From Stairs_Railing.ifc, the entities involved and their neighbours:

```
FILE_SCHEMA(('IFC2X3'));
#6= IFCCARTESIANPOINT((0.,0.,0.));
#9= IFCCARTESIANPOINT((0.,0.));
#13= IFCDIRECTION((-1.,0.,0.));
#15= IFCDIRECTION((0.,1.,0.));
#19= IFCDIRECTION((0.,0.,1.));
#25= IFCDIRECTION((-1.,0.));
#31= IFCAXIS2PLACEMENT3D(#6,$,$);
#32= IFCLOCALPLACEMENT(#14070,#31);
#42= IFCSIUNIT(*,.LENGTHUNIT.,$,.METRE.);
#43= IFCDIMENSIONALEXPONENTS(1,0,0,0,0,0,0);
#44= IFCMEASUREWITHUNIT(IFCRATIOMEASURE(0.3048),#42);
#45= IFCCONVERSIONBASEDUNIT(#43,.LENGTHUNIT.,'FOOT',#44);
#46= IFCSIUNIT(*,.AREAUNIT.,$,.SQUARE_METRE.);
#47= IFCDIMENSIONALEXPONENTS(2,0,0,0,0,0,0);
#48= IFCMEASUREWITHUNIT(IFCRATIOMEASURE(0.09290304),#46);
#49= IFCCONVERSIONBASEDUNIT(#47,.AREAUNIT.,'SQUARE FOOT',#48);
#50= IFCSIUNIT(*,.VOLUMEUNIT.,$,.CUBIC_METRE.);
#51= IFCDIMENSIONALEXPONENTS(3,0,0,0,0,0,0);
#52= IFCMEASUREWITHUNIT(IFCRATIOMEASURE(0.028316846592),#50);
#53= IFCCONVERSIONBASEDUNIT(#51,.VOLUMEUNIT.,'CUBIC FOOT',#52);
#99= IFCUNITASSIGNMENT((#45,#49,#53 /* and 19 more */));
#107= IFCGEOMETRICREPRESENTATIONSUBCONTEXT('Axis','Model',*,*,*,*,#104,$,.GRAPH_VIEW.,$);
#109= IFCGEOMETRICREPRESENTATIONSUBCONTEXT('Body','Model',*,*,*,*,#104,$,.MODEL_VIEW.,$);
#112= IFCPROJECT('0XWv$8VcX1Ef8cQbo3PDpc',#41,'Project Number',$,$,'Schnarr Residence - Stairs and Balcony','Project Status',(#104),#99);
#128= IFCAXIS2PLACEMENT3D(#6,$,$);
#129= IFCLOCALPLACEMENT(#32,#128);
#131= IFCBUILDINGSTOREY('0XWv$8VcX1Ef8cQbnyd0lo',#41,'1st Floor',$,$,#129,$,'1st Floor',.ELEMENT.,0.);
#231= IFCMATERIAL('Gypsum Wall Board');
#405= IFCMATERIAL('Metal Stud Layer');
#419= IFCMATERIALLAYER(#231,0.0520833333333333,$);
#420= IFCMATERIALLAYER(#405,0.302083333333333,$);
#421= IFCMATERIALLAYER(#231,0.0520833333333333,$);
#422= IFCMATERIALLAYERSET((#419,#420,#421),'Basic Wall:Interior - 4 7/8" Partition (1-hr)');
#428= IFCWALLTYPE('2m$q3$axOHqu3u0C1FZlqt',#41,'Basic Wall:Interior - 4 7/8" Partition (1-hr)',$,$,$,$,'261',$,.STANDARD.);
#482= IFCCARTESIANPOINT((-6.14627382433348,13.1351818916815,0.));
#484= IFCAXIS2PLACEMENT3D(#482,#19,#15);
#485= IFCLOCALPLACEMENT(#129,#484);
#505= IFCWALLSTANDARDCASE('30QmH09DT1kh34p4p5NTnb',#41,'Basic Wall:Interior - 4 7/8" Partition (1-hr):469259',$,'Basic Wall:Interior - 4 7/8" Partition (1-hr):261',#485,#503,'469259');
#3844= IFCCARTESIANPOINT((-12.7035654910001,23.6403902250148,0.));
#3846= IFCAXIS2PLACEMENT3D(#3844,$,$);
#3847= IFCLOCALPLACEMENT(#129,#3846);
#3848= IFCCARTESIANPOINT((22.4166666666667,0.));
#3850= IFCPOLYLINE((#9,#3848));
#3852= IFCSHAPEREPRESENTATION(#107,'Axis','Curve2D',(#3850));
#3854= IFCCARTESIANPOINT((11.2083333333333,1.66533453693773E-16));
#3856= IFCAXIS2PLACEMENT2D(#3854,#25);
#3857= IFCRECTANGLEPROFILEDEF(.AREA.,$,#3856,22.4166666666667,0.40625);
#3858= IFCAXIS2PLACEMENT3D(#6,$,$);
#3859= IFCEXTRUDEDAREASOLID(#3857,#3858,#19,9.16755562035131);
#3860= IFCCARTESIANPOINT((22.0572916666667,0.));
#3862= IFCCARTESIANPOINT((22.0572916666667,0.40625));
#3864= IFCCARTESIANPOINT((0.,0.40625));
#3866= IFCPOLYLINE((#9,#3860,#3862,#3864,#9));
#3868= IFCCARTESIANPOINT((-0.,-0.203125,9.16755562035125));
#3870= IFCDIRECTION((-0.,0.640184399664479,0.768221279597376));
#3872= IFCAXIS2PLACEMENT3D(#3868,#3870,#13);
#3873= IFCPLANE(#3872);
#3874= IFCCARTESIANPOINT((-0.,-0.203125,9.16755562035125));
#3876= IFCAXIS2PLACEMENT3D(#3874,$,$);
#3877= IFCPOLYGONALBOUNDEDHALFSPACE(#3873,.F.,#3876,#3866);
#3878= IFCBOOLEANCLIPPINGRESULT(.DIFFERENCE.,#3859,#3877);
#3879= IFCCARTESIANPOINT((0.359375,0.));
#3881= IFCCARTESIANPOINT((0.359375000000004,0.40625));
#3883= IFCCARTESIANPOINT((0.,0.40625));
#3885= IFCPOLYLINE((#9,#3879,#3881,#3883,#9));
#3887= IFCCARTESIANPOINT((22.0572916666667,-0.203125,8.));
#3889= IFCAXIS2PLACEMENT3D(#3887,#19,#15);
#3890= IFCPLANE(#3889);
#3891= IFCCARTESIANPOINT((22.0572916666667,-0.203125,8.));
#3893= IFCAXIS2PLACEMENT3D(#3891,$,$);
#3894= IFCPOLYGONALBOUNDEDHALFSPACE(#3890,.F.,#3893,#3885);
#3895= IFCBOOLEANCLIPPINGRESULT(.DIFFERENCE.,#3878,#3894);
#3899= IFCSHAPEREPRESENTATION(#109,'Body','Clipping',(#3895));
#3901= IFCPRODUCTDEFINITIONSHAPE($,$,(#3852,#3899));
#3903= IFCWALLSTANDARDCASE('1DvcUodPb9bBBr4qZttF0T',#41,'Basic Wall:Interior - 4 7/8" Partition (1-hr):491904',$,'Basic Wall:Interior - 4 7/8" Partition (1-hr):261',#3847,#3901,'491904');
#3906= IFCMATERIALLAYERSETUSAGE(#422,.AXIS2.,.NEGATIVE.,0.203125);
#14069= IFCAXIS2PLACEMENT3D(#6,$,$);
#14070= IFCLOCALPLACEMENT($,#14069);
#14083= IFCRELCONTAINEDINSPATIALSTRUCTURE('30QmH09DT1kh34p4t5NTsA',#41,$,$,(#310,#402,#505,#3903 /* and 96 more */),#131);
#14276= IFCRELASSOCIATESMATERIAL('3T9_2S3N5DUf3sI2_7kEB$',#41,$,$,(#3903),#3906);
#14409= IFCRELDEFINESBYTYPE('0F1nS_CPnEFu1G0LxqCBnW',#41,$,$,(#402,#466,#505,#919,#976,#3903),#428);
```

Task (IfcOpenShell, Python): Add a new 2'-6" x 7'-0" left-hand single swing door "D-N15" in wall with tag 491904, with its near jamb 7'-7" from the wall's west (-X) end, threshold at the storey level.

```python
import numpy as np
import ifcopenshell
import ifcopenshell.api.feature
import ifcopenshell.api.geometry
import ifcopenshell.api.root
import ifcopenshell.api.spatial
import ifcopenshell.api.type
import ifcopenshell.geom
import ifcopenshell.util.element
import ifcopenshell.util.placement
import ifcopenshell.util.representation
import ifcopenshell.util.shape
import ifcopenshell.util.unit

model = ifcopenshell.open("Stairs_Railing.ifc")
unit_scale = ifcopenshell.util.unit.calculate_unit_scale(model)
settings = ifcopenshell.geom.settings()


def volume(element):
    """Net volume in cubic metres, openings subtracted."""
    shape = ifcopenshell.geom.create_shape(settings, element)
    return ifcopenshell.util.shape.get_volume(shape.geometry)


wall = model.by_guid("1DvcUodPb9bBBr4qZttF0T")
storey = ifcopenshell.util.element.get_container(wall, ifc_class="IfcBuildingStorey")
context = ifcopenshell.util.representation.get_context(model, "Model", "Body", "MODEL_VIEW")
before = volume(wall)

width, height, from_end, sill = 0.762, 2.1336, 2.3114, 0.0  # metres

# The wall runs along its own X axis, and the end named is its -X end.
wall_shape = ifcopenshell.geom.create_shape(settings, wall)
x, y, z = ifcopenshell.util.shape.get_vertices(wall_shape.geometry).T
start = x.min() + from_end
face, thickness = float(y.min()), float(y.max() - y.min())
wall_matrix = ifcopenshell.util.placement.get_local_placement(wall.ObjectPlacement)
level = ifcopenshell.util.placement.get_local_placement(storey.ObjectPlacement)[2, 3]


def in_wall(x, y):
    """Placement at x, y metres in the wall's axes, at sill height."""
    matrix = wall_matrix.copy()
    matrix[:, 3] = wall_matrix @ np.array([x / unit_scale, y / unit_scale, 0.0, 1.0])
    matrix[2, 3] = level + sill / unit_scale
    return matrix


# Opening: a box that overshoots both wall faces by 50 mm.
opening = ifcopenshell.api.root.create_entity(model, ifc_class="IfcOpeningElement")
box = ifcopenshell.api.geometry.add_wall_representation(
    model, context=context, length=width, height=height, thickness=thickness + 0.1
)
ifcopenshell.api.geometry.assign_representation(model, product=opening, representation=box)
ifcopenshell.api.geometry.edit_object_placement(model, product=opening, matrix=in_wall(start, face - 0.05), is_si=False)
ifcopenshell.api.feature.add_feature(model, feature=opening, element=wall)

door = ifcopenshell.api.root.create_entity(model, ifc_class="IfcDoor", name="D-N15")
door.OverallWidth, door.OverallHeight = width / unit_scale, height / unit_scale
body = ifcopenshell.api.geometry.add_door_representation(
    model,
    context=context,
    overall_width=door.OverallWidth,
    overall_height=door.OverallHeight,
    operation_type="SINGLE_SWING_LEFT",
    lining_properties={"LiningDepth": thickness / unit_scale, "ThresholdDepth": thickness / unit_scale},
)
ifcopenshell.api.geometry.assign_representation(model, product=door, representation=body)
ifcopenshell.api.spatial.assign_container(model, products=[door], relating_structure=storey)
fills = ifcopenshell.api.feature.add_filling(model, opening=opening, element=door)
fills.OwnerHistory = door.OwnerHistory  # required in IFC2X3

# IFC2X3 keeps the operation on the door style.
style = ifcopenshell.api.root.create_entity(model, ifc_class="IfcDoorStyle", name="D-N15")
style.OperationType, style.ConstructionType = "SINGLE_SWING_LEFT", "NOTDEFINED"
style.ParameterTakesPrecedence = style.Sizeable = False
ifcopenshell.api.type.assign_type(model, related_objects=[door], relating_type=style)

# The lining spans the wall, so the door starts at the wall face.
ifcopenshell.api.geometry.edit_object_placement(model, product=door, matrix=in_wall(start, face), is_si=False)

after = volume(wall)

print(f"wall volume {before:.3f} -> {after:.3f} m3")

model.write("Stairs_Railing_rev.ifc")
```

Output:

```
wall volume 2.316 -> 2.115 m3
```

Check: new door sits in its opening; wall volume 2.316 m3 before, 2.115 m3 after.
